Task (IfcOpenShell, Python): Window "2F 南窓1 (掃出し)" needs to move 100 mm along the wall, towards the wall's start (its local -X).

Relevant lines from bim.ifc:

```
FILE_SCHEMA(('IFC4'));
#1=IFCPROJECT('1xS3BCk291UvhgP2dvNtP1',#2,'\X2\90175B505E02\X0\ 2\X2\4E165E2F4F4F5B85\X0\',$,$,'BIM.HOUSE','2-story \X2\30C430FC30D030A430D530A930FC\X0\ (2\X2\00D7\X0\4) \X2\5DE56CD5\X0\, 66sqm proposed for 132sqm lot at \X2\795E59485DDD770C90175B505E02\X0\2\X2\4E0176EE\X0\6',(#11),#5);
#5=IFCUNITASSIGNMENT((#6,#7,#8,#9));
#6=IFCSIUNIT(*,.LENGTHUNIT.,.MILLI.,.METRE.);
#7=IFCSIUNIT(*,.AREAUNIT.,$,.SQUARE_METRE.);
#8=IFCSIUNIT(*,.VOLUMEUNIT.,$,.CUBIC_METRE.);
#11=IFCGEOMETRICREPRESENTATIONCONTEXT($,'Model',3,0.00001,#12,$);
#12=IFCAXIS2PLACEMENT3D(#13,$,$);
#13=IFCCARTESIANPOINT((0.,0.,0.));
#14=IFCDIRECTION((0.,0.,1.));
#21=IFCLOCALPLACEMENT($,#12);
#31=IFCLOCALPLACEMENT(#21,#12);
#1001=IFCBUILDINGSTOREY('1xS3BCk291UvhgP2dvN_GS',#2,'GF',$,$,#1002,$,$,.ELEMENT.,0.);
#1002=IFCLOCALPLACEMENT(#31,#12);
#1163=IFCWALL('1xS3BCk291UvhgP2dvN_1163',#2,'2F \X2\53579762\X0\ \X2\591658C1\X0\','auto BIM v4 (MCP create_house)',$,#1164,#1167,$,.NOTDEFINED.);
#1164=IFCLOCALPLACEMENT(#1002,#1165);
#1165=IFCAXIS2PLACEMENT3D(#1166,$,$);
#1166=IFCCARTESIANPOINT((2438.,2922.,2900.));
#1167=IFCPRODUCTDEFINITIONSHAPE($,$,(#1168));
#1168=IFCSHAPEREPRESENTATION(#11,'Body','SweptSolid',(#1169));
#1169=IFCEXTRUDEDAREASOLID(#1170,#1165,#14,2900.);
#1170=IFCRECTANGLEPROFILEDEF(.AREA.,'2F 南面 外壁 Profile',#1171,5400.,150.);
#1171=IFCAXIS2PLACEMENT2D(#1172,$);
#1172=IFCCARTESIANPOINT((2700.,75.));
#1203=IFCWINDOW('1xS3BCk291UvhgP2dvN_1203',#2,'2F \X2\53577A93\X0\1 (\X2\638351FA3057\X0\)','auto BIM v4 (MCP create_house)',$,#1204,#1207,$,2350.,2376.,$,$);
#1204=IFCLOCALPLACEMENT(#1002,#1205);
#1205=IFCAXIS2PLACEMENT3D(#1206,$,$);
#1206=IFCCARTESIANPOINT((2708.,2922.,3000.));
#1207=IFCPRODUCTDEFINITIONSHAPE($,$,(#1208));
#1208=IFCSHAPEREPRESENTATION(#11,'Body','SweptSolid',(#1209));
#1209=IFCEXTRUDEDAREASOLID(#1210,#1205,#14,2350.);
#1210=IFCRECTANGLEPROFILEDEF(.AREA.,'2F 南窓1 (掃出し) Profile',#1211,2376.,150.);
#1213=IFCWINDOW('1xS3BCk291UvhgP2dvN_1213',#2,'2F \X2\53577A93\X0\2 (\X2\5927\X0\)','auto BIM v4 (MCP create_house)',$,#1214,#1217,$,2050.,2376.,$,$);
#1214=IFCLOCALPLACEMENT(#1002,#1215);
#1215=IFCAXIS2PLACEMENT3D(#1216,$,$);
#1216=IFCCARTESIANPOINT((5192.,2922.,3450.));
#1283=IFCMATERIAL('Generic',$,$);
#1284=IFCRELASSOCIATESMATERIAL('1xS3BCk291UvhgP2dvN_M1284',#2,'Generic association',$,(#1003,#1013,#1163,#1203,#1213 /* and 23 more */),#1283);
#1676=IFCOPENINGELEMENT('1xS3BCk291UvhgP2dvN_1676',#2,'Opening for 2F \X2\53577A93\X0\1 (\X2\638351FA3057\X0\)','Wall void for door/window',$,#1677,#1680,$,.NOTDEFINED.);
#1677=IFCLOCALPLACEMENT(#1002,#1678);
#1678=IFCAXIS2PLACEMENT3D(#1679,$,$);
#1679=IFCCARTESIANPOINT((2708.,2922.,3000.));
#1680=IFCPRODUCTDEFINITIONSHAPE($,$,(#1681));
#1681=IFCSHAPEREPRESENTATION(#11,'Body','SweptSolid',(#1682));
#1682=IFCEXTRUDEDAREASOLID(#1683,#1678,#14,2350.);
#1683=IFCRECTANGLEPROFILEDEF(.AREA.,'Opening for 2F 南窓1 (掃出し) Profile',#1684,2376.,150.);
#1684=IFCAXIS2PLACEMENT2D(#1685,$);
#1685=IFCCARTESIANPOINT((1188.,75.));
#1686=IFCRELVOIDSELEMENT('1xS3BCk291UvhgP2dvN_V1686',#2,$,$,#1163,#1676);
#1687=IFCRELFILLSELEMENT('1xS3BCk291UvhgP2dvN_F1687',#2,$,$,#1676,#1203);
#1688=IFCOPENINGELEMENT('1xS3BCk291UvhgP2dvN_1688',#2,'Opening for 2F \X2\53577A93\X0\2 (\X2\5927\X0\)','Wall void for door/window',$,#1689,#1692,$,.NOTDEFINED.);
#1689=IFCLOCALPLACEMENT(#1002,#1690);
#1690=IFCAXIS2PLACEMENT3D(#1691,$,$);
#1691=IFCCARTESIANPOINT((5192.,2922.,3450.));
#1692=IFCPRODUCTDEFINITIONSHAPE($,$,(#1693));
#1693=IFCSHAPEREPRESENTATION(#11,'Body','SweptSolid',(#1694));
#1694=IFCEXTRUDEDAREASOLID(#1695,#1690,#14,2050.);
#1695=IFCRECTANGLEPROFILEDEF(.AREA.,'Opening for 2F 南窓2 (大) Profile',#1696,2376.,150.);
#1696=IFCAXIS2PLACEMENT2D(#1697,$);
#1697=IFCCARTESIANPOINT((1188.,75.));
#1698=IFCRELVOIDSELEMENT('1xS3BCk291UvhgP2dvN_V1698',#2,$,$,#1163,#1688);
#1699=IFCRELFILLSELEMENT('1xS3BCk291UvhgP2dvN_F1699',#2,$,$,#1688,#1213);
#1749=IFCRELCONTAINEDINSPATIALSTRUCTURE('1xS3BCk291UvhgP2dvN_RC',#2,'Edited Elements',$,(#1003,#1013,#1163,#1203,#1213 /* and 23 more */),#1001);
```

```python
import ifcopenshell
import ifcopenshell.api.geometry
import ifcopenshell.util.placement
import ifcopenshell.util.unit

model = ifcopenshell.open("bim.ifc")
unit_scale = ifcopenshell.util.unit.calculate_unit_scale(model)

window = model.by_id(1203)
opening = window.FillsVoids[0].RelatingOpeningElement
wall = opening.VoidsElements[0].RelatingBuildingElement

wall_matrix = ifcopenshell.util.placement.get_local_placement(wall.ObjectPlacement)
shift = wall_matrix[:3, 0] * -0.1 / unit_scale
before = ifcopenshell.util.placement.get_local_placement(window.ObjectPlacement)[:3, 3].copy()

# The window is not placed relative to its opening, so move both.
for product in (opening, window):
    matrix = ifcopenshell.util.placement.get_local_placement(product.ObjectPlacement)
    matrix[:3, 3] += shift
    ifcopenshell.api.geometry.edit_object_placement(model, product=product, matrix=matrix, is_si=False)

after = ifcopenshell.util.placement.get_local_placement(window.ObjectPlacement)[:3, 3]
print("window moved by", (after - before).round(3) + 0.0)

model.write("bim_v2.ifc")
```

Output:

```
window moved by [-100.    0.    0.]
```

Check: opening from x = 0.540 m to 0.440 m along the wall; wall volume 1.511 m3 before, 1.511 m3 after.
